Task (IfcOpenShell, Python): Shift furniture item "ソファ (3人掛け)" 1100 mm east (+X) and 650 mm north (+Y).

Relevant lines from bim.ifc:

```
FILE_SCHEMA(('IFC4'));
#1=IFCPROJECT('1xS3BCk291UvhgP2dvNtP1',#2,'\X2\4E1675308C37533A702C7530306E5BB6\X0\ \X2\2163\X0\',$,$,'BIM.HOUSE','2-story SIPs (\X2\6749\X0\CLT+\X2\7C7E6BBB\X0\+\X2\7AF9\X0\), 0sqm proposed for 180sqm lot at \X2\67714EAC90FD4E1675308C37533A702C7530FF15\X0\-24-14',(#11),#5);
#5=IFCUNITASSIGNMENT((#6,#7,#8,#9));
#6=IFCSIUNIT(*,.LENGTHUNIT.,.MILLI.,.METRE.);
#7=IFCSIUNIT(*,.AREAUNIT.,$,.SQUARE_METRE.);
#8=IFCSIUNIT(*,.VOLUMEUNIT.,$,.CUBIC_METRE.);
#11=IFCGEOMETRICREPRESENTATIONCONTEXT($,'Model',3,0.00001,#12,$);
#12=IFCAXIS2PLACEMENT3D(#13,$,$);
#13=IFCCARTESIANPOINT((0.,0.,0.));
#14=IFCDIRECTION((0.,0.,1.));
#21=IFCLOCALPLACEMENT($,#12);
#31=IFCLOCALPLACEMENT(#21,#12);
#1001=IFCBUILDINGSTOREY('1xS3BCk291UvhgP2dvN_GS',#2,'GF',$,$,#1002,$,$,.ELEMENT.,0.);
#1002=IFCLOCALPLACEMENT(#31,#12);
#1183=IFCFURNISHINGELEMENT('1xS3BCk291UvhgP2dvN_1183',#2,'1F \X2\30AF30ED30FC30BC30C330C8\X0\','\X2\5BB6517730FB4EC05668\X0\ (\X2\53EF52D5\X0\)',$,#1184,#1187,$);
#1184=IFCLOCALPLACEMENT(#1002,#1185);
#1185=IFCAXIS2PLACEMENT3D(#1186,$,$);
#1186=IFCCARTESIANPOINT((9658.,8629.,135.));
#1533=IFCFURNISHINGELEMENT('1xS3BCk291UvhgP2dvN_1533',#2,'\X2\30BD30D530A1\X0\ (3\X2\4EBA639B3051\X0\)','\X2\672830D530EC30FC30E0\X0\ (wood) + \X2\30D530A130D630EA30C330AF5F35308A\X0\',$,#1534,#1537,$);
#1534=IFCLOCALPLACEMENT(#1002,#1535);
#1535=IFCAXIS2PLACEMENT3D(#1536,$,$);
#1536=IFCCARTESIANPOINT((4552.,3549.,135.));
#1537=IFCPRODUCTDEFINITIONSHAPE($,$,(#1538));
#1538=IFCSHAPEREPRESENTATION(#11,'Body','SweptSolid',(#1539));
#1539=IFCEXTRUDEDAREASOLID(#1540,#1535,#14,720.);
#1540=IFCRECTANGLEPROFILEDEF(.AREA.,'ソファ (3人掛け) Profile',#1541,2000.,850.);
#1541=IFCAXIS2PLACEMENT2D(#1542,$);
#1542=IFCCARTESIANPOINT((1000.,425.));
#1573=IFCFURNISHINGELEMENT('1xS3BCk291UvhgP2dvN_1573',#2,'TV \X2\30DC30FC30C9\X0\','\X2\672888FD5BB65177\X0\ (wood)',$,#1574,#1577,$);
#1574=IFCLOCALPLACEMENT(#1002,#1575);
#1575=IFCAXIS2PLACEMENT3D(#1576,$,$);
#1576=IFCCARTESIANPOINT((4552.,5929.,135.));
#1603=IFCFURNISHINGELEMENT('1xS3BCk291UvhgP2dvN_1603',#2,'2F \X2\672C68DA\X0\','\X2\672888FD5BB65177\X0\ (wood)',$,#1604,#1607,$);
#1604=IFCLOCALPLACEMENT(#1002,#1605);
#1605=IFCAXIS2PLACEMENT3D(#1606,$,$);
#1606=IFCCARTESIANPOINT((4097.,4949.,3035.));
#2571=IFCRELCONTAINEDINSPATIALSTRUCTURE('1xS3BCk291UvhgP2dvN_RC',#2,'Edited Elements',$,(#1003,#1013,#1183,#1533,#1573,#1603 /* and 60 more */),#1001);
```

```python
import ifcopenshell
import ifcopenshell.api.geometry
import ifcopenshell.util.placement

model = ifcopenshell.open("bim.ifc")

item = model.by_id(1533)
matrix = ifcopenshell.util.placement.get_local_placement(item.ObjectPlacement)
matrix[0, 3] += 1100.0
matrix[1, 3] += 650.0
ifcopenshell.api.geometry.edit_object_placement(model, product=item, matrix=matrix, is_si=False)

print(ifcopenshell.util.placement.get_local_placement(item.ObjectPlacement).round(3) + 0.0)

model.write("bim_rev.ifc")
```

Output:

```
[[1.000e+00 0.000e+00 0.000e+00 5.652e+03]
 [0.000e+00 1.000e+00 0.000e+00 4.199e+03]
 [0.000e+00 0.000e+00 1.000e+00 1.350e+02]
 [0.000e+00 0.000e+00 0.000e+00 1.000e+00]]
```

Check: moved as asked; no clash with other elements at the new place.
